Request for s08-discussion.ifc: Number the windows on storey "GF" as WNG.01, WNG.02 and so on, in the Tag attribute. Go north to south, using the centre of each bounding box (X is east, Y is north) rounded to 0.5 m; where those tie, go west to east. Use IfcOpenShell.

First a look at what the model holds.

```python
import ifcopenshell
import ifcopenshell.util.element
import ifcopenshell.util.placement

model = ifcopenshell.open("s08-discussion.ifc")
print(model.schema)
storey = next(s for s in model.by_type("IfcBuildingStorey") if s.Name == "GF")
windows = [e for e in ifcopenshell.util.element.get_decomposition(storey) if e.is_a("IfcWindow")]
for e in sorted(windows, key=lambda e: e.id()):
    origin = ifcopenshell.util.placement.get_local_placement(e.ObjectPlacement)[:3, 3]
    print(e.id(), e.Tag, e.Name, origin.round(2) + 0.0, sep=" | ")
```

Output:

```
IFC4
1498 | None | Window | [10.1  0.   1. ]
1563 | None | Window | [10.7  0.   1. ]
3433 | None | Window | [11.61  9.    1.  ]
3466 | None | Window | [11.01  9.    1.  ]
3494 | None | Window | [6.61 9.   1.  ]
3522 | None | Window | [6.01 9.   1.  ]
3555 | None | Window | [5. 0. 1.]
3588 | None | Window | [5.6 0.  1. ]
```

```python
import ifcopenshell
import ifcopenshell.geom
import ifcopenshell.util.element
import ifcopenshell.util.shape

model = ifcopenshell.open("s08-discussion.ifc")
settings = ifcopenshell.geom.settings()
settings.set("use-world-coords", True)


def centre(element):
    shape = ifcopenshell.geom.create_shape(settings, element)
    return ifcopenshell.util.shape.get_bbox_centroid(shape.geometry)


storey = next(s for s in model.by_type("IfcBuildingStorey") if s.Name == "GF")
windows = [e for e in ifcopenshell.util.element.get_decomposition(storey) if e.is_a("IfcWindow")]

# Insertion points can sit at a corner or the storey origin, so sort by the geometry (in metres).
centres = {e: centre(e) for e in windows}
windows.sort(key=lambda e: (-round(centres[e][1] / 0.5), centres[e][0]))

for i, e in enumerate(windows, start=1):
    number = f"WNG.{i:02d}"
    e.Tag = number
    print(e.id(), number)

model.write("s08-discussion_updated.ifc")
```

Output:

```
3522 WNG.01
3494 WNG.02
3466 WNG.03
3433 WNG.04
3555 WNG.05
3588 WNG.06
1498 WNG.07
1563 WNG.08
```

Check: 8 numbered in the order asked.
